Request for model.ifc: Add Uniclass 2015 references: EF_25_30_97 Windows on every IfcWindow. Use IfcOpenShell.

First a look at what the model holds.

```python
import ifcopenshell

model = ifcopenshell.open("model.ifc")
print(model.schema)
print("classifications:", [c.Name for c in model.by_type("IfcClassification")])
for ifc_class in ("IfcDoor", "IfcRoof", "IfcStair", "IfcWall", "IfcWindow"):
    print(ifc_class, len(model.by_type(ifc_class)))
```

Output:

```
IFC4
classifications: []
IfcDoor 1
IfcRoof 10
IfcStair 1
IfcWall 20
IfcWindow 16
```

```python
import ifcopenshell
import ifcopenshell.api.classification

model = ifcopenshell.open("model.ifc")

system = ifcopenshell.api.classification.add_classification(model, classification="Uniclass 2015")

codes = {
    "IfcWindow": ("EF_25_30_97", "Windows"),
}
for ifc_class, (code, name) in codes.items():
    products = model.by_type(ifc_class)
    ifcopenshell.api.classification.add_reference(
        model, products=products, classification=system, identification=code, name=name
    )
    print(code, len(products))

model.write("model_updated.ifc")
```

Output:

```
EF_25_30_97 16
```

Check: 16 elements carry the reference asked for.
